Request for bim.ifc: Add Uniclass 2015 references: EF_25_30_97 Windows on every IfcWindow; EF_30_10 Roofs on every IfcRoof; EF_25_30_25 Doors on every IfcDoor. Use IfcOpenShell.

First a look at what the model holds.

```python
import ifcopenshell

model = ifcopenshell.open("bim.ifc")
print(model.schema)
print("classifications:", [c.Name for c in model.by_type("IfcClassification")])
for ifc_class in ("IfcDoor", "IfcRoof", "IfcStair", "IfcWall", "IfcWindow"):
    print(ifc_class, len(model.by_type(ifc_class)))
```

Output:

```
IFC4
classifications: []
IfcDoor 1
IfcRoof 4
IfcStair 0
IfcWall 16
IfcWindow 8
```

```python
import ifcopenshell
import ifcopenshell.api.classification

model = ifcopenshell.open("bim.ifc")

system = ifcopenshell.api.classification.add_classification(model, classification="Uniclass 2015")

codes = {
    "IfcWindow": ("EF_25_30_97", "Windows"),
    "IfcRoof": ("EF_30_10", "Roofs"),
    "IfcDoor": ("EF_25_30_25", "Doors"),
}
for ifc_class, (code, name) in codes.items():
    products = model.by_type(ifc_class)
    ifcopenshell.api.classification.add_reference(
        model, products=products, classification=system, identification=code, name=name
    )
    print(code, len(products))

model.write("bim_rev.ifc")
```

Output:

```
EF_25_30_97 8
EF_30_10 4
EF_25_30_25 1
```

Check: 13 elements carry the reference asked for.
